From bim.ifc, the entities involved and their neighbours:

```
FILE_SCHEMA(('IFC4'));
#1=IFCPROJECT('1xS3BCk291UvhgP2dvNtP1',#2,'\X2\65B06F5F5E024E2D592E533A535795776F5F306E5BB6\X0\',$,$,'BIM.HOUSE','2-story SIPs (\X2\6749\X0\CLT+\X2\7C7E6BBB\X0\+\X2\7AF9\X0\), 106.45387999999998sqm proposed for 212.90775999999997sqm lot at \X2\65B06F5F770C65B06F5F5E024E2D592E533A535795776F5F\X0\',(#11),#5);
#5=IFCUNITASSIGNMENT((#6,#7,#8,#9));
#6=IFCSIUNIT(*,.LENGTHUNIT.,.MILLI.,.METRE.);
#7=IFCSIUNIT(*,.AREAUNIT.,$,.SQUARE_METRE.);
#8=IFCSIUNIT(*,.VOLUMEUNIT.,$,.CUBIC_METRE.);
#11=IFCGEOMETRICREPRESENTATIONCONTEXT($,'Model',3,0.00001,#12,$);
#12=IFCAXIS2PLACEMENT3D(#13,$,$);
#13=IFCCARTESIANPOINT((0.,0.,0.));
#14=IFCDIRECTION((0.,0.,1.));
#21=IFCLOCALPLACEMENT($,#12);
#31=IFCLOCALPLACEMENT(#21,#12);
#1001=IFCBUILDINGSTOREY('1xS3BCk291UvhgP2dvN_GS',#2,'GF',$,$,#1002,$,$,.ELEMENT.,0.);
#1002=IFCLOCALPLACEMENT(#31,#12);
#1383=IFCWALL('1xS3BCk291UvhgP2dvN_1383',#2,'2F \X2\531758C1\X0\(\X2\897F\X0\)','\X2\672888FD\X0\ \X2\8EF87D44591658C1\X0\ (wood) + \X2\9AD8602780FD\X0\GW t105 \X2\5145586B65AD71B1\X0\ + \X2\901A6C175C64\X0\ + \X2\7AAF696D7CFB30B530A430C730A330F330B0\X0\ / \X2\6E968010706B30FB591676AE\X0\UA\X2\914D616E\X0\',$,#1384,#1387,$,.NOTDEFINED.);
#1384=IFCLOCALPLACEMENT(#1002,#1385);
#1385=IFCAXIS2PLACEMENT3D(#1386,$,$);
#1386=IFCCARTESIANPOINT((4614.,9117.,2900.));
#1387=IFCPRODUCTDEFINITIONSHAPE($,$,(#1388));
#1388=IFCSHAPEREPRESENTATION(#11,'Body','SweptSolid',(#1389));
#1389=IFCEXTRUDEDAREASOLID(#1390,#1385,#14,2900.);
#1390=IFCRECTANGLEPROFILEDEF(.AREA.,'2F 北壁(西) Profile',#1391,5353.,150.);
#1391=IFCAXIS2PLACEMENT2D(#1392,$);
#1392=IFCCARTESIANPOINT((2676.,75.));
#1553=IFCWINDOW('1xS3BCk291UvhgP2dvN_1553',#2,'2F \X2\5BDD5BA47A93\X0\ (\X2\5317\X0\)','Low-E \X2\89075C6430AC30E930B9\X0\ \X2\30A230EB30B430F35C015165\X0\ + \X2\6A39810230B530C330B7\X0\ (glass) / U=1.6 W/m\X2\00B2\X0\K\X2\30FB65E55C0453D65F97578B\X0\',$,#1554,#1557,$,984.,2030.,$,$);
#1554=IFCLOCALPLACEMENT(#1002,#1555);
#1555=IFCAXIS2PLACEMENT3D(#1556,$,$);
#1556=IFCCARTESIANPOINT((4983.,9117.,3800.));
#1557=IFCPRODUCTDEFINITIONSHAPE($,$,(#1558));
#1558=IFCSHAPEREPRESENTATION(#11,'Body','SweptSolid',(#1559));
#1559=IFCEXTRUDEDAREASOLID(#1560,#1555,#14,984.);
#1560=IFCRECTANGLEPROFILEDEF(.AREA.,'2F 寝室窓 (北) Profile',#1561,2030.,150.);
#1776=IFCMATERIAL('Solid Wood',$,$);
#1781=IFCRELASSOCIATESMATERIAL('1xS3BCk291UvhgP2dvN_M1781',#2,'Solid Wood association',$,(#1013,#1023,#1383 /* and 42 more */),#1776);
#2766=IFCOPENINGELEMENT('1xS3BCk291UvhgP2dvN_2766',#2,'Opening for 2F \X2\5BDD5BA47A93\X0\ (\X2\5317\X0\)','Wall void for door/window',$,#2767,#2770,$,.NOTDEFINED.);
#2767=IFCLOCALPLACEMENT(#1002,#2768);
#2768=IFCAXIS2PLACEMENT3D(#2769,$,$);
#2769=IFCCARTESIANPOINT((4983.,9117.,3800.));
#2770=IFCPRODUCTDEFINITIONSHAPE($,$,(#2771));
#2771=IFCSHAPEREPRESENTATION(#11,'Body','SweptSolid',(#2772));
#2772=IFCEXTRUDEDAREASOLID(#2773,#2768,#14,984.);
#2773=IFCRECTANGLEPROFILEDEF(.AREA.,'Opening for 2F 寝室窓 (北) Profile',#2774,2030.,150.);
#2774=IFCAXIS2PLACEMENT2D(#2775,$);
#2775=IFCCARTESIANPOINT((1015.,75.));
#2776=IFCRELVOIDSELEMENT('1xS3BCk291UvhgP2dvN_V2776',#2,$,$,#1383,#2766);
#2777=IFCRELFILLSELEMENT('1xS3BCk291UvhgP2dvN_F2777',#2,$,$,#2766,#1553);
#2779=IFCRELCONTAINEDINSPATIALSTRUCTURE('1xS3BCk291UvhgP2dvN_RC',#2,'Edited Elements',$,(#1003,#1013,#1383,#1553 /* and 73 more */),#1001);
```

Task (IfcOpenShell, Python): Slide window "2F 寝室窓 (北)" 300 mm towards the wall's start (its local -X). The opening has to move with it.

```python
import ifcopenshell
import ifcopenshell.api.geometry
import ifcopenshell.util.placement

model = ifcopenshell.open("bim.ifc")

window = model.by_id(1553)
opening = window.FillsVoids[0].RelatingOpeningElement
wall = opening.VoidsElements[0].RelatingBuildingElement

wall_matrix = ifcopenshell.util.placement.get_local_placement(wall.ObjectPlacement)
shift = wall_matrix[:3, 0] * -300.0
before = ifcopenshell.util.placement.get_local_placement(window.ObjectPlacement)[:3, 3].copy()

# The window is not placed relative to its opening, so move both.
for product in (opening, window):
    matrix = ifcopenshell.util.placement.get_local_placement(product.ObjectPlacement)
    matrix[:3, 3] += shift
    ifcopenshell.api.geometry.edit_object_placement(model, product=product, matrix=matrix, is_si=False)

after = ifcopenshell.util.placement.get_local_placement(window.ObjectPlacement)[:3, 3]
print("window moved by", (after - before).round(3) + 0.0)

model.write("bim_v2.ifc")
```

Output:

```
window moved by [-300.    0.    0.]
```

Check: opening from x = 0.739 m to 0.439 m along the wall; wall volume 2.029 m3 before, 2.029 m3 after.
